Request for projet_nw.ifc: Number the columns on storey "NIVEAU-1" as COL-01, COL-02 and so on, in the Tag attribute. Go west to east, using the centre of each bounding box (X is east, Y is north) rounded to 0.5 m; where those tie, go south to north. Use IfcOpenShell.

First a look at what the model holds.

```python
import ifcopenshell
import ifcopenshell.util.element
import ifcopenshell.util.placement

model = ifcopenshell.open("projet_nw.ifc")
print(model.schema)
storey = next(s for s in model.by_type("IfcBuildingStorey") if s.Name == "NIVEAU-1")
columns = [e for e in ifcopenshell.util.element.get_decomposition(storey) if e.is_a("IfcColumn")]
for e in sorted(columns, key=lambda e: e.id()):
    origin = ifcopenshell.util.placement.get_local_placement(e.ObjectPlacement)[:3, 3]
    print(e.id(), e.Tag, e.Name, origin.round(2) + 0.0, sep=" | ")
```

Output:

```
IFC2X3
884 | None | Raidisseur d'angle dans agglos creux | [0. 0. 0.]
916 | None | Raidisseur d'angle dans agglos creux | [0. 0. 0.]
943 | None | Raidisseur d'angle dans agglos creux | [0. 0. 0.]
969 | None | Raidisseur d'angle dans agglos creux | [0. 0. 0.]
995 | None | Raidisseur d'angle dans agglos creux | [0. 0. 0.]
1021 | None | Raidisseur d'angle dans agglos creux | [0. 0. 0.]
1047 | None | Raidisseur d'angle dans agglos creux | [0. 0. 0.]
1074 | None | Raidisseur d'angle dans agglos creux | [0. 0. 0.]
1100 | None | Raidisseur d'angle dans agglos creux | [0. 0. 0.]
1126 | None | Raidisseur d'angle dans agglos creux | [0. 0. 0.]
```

```python
import ifcopenshell
import ifcopenshell.geom
import ifcopenshell.util.element
import ifcopenshell.util.shape

model = ifcopenshell.open("projet_nw.ifc")
settings = ifcopenshell.geom.settings()
settings.set("use-world-coords", True)


def centre(element):
    shape = ifcopenshell.geom.create_shape(settings, element)
    return ifcopenshell.util.shape.get_bbox_centroid(shape.geometry)


storey = next(s for s in model.by_type("IfcBuildingStorey") if s.Name == "NIVEAU-1")
columns = [e for e in ifcopenshell.util.element.get_decomposition(storey) if e.is_a("IfcColumn")]

# Insertion points can sit at a corner or the storey origin, so sort by the geometry (in metres).
centres = {e: centre(e) for e in columns}
columns.sort(key=lambda e: (round(centres[e][0] / 0.5), centres[e][1]))

for i, e in enumerate(columns, start=1):
    number = f"COL-{i:02d}"
    e.Tag = number
    print(e.id(), number)

model.write("projet_nw_rev.ifc")
```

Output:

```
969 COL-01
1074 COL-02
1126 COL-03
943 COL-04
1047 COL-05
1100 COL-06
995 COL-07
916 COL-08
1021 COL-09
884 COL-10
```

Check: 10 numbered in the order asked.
